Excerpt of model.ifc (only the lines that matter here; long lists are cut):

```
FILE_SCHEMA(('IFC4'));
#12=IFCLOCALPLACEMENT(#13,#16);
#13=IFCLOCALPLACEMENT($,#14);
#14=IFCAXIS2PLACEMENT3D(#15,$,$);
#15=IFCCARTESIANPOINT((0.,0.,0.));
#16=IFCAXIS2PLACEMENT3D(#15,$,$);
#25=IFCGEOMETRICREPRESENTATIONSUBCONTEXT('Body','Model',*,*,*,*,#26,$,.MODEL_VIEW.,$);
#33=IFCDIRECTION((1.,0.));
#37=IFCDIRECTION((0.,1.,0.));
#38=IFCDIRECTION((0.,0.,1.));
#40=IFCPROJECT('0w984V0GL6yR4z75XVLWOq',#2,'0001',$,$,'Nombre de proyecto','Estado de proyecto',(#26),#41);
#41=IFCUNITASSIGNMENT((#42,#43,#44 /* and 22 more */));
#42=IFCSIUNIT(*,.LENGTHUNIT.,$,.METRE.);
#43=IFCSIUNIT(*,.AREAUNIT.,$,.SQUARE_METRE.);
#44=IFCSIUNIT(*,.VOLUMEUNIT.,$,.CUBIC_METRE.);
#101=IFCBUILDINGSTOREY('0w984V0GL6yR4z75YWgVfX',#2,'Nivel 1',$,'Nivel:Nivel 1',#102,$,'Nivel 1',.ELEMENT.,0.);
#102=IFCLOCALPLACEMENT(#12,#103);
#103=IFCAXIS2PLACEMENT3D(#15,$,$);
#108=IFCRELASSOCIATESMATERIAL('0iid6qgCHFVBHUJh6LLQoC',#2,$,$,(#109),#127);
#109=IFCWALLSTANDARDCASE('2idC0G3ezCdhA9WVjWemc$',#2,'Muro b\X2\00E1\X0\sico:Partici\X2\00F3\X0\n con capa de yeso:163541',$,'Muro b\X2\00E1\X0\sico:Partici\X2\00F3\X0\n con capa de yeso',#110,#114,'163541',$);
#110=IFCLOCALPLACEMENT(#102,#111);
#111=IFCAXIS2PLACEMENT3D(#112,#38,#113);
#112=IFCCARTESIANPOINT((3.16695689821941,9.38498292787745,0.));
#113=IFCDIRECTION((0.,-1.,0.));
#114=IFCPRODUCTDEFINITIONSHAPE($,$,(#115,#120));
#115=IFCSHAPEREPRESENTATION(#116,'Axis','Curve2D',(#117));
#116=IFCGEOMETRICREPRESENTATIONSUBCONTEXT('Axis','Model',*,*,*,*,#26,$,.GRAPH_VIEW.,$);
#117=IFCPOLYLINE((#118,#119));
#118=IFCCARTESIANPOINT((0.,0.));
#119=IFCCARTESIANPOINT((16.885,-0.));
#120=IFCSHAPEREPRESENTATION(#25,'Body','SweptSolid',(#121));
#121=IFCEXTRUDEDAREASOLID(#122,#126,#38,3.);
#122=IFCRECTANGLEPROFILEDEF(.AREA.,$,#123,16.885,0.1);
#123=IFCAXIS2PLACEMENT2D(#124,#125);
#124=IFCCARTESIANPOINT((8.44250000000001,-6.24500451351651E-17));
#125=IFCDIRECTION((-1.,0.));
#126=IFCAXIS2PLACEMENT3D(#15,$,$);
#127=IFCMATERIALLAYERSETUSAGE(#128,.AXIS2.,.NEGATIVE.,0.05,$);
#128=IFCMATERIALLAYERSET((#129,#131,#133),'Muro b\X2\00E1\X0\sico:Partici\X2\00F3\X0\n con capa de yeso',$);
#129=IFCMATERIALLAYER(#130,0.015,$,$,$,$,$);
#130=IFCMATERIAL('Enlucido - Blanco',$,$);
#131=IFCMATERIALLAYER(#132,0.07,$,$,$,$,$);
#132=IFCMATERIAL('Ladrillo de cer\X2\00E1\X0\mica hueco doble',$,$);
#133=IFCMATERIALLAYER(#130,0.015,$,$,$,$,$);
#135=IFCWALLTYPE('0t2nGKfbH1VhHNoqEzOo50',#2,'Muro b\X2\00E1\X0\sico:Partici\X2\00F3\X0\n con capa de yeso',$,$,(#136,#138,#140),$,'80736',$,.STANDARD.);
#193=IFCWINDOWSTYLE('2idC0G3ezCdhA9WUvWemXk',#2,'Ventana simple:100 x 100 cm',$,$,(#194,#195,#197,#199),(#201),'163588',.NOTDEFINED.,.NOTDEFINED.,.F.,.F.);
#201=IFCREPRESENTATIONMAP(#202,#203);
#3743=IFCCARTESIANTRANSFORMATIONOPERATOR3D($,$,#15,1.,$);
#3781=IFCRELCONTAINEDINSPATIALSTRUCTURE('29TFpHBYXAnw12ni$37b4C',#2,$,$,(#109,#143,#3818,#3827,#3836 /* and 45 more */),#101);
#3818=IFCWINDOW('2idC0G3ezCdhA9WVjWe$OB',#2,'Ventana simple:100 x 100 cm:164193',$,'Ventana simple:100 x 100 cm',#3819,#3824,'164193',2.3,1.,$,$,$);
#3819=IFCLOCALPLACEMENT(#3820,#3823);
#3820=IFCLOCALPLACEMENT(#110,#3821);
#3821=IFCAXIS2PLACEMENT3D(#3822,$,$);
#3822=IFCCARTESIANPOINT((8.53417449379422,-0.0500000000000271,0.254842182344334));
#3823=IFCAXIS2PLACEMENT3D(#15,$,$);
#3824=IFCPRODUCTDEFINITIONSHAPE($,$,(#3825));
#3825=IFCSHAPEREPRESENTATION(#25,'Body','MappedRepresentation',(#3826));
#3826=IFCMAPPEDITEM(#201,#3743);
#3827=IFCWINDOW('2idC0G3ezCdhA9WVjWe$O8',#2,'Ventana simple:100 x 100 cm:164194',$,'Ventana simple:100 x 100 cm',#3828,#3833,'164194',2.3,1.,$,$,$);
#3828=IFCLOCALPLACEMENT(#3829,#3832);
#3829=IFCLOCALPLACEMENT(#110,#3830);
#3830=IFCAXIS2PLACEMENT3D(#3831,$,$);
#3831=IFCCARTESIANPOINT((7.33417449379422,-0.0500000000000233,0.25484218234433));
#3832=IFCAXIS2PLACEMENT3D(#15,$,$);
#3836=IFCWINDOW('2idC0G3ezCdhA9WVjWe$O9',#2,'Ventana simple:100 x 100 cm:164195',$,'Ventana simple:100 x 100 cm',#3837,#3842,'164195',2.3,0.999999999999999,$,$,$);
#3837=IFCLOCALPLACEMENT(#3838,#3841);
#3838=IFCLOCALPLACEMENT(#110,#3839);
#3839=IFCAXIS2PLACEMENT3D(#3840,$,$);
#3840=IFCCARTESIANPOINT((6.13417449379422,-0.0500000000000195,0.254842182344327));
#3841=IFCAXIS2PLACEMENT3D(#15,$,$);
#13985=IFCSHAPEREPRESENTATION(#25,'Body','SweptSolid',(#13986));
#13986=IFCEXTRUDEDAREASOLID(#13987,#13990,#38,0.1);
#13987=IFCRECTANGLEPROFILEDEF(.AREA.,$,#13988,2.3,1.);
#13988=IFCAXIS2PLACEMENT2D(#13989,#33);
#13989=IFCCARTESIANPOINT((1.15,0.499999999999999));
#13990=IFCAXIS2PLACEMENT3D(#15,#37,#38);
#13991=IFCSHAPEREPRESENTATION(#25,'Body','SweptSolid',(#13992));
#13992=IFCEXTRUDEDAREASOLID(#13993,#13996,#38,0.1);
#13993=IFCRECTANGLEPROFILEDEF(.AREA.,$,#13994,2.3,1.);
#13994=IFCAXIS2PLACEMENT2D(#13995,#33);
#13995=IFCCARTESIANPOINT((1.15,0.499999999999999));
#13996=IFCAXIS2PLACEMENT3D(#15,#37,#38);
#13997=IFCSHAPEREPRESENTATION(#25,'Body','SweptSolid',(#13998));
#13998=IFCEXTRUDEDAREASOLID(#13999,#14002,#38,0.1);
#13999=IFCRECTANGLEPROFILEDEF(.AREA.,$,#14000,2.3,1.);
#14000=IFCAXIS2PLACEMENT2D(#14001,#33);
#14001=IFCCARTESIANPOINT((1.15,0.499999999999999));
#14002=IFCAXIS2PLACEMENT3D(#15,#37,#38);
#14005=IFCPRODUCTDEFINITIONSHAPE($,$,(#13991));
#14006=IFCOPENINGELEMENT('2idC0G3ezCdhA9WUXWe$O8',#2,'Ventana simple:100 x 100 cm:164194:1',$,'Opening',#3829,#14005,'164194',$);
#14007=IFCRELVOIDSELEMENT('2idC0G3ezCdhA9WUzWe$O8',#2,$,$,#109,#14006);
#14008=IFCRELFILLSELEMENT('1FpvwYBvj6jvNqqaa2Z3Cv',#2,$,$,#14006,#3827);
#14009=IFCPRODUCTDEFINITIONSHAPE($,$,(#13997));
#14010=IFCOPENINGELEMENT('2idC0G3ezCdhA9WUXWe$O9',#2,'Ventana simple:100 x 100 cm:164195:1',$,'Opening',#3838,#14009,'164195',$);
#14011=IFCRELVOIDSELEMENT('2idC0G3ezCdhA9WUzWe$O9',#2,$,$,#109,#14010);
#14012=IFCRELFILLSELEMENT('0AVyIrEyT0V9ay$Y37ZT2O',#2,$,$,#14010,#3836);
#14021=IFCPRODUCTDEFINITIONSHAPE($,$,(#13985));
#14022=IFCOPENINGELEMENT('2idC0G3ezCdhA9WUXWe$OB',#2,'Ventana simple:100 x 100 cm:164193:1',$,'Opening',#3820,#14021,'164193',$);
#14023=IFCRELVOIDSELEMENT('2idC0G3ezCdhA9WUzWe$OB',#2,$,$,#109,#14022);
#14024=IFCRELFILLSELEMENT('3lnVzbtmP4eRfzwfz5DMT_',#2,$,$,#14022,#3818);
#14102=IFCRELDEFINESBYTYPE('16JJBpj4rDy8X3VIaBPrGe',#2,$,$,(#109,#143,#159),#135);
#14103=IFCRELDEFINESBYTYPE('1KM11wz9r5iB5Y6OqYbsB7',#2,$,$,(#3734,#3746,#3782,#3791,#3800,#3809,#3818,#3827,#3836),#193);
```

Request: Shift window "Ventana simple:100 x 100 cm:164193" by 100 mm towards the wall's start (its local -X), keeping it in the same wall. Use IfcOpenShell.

```python
import ifcopenshell
import ifcopenshell.api.geometry
import ifcopenshell.util.placement

model = ifcopenshell.open("model.ifc")

window = model.by_id(3818)
opening = window.FillsVoids[0].RelatingOpeningElement
wall = opening.VoidsElements[0].RelatingBuildingElement

wall_matrix = ifcopenshell.util.placement.get_local_placement(wall.ObjectPlacement)
shift = wall_matrix[:3, 0] * -0.1
before = ifcopenshell.util.placement.get_local_placement(window.ObjectPlacement)[:3, 3].copy()

# The window is placed relative to its opening, so it follows when the opening moves.
matrix = ifcopenshell.util.placement.get_local_placement(opening.ObjectPlacement)
matrix[:3, 3] += shift
ifcopenshell.api.geometry.edit_object_placement(
    model, product=opening, matrix=matrix, is_si=False, should_transform_children=True
)

after = ifcopenshell.util.placement.get_local_placement(window.ObjectPlacement)[:3, 3]
print("window moved by", (after - before).round(3) + 0.0)

model.write("model_v2.ifc")
```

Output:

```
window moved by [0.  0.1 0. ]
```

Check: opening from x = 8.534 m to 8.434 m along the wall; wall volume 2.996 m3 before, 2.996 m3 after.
